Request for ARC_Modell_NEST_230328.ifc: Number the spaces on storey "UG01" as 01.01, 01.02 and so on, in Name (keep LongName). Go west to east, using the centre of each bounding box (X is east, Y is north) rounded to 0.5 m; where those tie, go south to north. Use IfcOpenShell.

First a look at what the model holds.

```python
import ifcopenshell
import ifcopenshell.util.element
import ifcopenshell.util.placement

model = ifcopenshell.open("ARC_Modell_NEST_230328.ifc")
print(model.schema)
storey = next(s for s in model.by_type("IfcBuildingStorey") if s.Name == "UG01")
spaces = [e for e in ifcopenshell.util.element.get_decomposition(storey) if e.is_a("IfcSpace")]
for e in sorted(spaces, key=lambda e: e.id()):
    origin = ifcopenshell.util.placement.get_local_placement(e.ObjectPlacement)[:3, 3]
    print(e.id(), e.Name, e.LongName, origin.round(2) + 0.0, sep=" | ")
```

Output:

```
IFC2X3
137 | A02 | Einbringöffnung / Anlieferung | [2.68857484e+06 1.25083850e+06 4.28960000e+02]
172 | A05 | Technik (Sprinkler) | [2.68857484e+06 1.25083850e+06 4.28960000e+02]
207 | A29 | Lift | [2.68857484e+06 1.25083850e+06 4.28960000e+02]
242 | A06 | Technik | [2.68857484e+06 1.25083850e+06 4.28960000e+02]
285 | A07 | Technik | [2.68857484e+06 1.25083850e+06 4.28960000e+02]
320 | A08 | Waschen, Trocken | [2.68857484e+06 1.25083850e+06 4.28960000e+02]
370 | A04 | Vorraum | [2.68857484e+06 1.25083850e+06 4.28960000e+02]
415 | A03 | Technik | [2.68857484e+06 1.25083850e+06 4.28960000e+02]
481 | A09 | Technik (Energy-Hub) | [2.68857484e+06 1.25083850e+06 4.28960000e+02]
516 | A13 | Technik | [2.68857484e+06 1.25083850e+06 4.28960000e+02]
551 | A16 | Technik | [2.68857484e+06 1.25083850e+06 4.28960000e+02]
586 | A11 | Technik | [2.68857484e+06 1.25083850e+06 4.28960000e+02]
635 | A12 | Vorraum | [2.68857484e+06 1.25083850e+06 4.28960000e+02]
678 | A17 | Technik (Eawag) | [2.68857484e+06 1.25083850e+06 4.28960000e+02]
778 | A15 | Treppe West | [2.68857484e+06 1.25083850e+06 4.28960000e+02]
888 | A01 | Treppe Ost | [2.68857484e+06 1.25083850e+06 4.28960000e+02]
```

```python
import ifcopenshell
import ifcopenshell.geom
import ifcopenshell.util.element
import ifcopenshell.util.shape

model = ifcopenshell.open("ARC_Modell_NEST_230328.ifc")
settings = ifcopenshell.geom.settings()
settings.set("use-world-coords", True)


def centre(element):
    shape = ifcopenshell.geom.create_shape(settings, element)
    return ifcopenshell.util.shape.get_bbox_centroid(shape.geometry)


storey = next(s for s in model.by_type("IfcBuildingStorey") if s.Name == "UG01")
spaces = [e for e in ifcopenshell.util.element.get_decomposition(storey) if e.is_a("IfcSpace")]

# Insertion points can sit at a corner or the storey origin, so sort by the geometry (in metres).
centres = {e: centre(e) for e in spaces}
spaces.sort(key=lambda e: (round(centres[e][0] / 0.5), centres[e][1]))

for i, e in enumerate(spaces, start=1):
    number = f"01.{i:02d}"
    e.Name = number
    print(e.id(), number)

model.write("ARC_Modell_NEST_230328_v2.ifc")
```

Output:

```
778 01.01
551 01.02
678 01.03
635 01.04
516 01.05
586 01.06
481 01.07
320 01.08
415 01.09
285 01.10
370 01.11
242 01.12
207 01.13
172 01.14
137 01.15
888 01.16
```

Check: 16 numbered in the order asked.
